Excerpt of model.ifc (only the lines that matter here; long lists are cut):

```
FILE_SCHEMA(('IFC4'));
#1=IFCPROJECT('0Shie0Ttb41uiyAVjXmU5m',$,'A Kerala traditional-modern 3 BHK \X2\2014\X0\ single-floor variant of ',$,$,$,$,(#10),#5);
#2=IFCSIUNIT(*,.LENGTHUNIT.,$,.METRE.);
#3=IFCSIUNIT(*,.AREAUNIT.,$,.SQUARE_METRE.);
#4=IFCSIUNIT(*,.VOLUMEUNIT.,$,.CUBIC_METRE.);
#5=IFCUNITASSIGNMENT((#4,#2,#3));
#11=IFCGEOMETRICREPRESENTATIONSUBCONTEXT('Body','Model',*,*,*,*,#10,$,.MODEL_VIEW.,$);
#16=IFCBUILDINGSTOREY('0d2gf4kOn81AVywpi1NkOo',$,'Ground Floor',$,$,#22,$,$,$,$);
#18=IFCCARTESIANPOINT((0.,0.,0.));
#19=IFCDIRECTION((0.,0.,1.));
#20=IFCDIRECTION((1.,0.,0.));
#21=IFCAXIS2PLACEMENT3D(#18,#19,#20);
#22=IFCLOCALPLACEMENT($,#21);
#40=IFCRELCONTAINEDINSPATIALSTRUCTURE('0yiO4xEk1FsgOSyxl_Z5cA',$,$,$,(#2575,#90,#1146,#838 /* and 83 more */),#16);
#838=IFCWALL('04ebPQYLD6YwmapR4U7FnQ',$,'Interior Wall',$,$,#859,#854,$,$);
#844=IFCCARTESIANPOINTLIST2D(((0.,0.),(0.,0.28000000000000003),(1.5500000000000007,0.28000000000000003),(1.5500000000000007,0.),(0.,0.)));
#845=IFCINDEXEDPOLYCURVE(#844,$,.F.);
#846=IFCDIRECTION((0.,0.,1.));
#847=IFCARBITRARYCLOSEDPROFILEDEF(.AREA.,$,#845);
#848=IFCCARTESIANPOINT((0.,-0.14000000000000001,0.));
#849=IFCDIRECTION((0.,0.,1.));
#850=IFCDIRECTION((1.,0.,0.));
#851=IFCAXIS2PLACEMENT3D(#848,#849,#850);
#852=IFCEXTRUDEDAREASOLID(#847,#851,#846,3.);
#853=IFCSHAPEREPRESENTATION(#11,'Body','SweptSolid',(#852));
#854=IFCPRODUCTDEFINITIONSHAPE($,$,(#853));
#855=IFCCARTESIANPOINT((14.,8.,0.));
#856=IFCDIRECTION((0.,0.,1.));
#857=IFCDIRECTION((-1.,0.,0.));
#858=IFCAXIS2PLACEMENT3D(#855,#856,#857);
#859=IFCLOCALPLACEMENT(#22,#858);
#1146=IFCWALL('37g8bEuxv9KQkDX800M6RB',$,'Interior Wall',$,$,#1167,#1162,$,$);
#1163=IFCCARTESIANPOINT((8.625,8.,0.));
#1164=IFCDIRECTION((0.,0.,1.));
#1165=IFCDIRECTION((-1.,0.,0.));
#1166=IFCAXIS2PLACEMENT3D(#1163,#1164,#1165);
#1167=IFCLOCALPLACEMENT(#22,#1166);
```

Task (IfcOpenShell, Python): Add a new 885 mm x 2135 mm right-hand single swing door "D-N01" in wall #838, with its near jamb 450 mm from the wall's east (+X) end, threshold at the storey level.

```python
import numpy as np
import ifcopenshell
import ifcopenshell.api.feature
import ifcopenshell.api.geometry
import ifcopenshell.api.root
import ifcopenshell.api.spatial
import ifcopenshell.geom
import ifcopenshell.util.element
import ifcopenshell.util.placement
import ifcopenshell.util.representation
import ifcopenshell.util.shape
import ifcopenshell.util.unit

model = ifcopenshell.open("model.ifc")
unit_scale = ifcopenshell.util.unit.calculate_unit_scale(model)
settings = ifcopenshell.geom.settings()


def volume(element):
    """Net volume in cubic metres, openings subtracted."""
    shape = ifcopenshell.geom.create_shape(settings, element)
    return ifcopenshell.util.shape.get_volume(shape.geometry)


wall = model.by_guid("04ebPQYLD6YwmapR4U7FnQ")
storey = ifcopenshell.util.element.get_container(wall, ifc_class="IfcBuildingStorey")
context = ifcopenshell.util.representation.get_context(model, "Model", "Body", "MODEL_VIEW")
before = volume(wall)

width, height, from_end, sill = 0.885, 2.135, 0.45, 0.0  # metres

# The wall runs along its own X axis, and the end named is its -X end.
wall_shape = ifcopenshell.geom.create_shape(settings, wall)
x, y, z = ifcopenshell.util.shape.get_vertices(wall_shape.geometry).T
start = x.min() + from_end
face, thickness = float(y.min()), float(y.max() - y.min())
wall_matrix = ifcopenshell.util.placement.get_local_placement(wall.ObjectPlacement)
level = ifcopenshell.util.placement.get_local_placement(storey.ObjectPlacement)[2, 3]


def in_wall(x, y):
    """Placement at x, y metres in the wall's axes, at sill height."""
    matrix = wall_matrix.copy()
    matrix[:, 3] = wall_matrix @ np.array([x / unit_scale, y / unit_scale, 0.0, 1.0])
    matrix[2, 3] = level + sill / unit_scale
    return matrix


# Opening: a box that overshoots both wall faces by 50 mm.
opening = ifcopenshell.api.root.create_entity(model, ifc_class="IfcOpeningElement", predefined_type="OPENING")
box = ifcopenshell.api.geometry.add_wall_representation(
    model, context=context, length=width, height=height, thickness=thickness + 0.1
)
ifcopenshell.api.geometry.assign_representation(model, product=opening, representation=box)
ifcopenshell.api.geometry.edit_object_placement(model, product=opening, matrix=in_wall(start, face - 0.05), is_si=False)
ifcopenshell.api.feature.add_feature(model, feature=opening, element=wall)

door = ifcopenshell.api.root.create_entity(model, ifc_class="IfcDoor", name="D-N01", predefined_type="DOOR")
door.OverallWidth, door.OverallHeight = width / unit_scale, height / unit_scale
door.OperationType = "SINGLE_SWING_RIGHT"
body = ifcopenshell.api.geometry.add_door_representation(
    model,
    context=context,
    overall_width=door.OverallWidth,
    overall_height=door.OverallHeight,
    operation_type="SINGLE_SWING_RIGHT",
    lining_properties={"LiningDepth": thickness / unit_scale, "ThresholdDepth": thickness / unit_scale},
)
ifcopenshell.api.geometry.assign_representation(model, product=door, representation=body)
ifcopenshell.api.spatial.assign_container(model, products=[door], relating_structure=storey)
ifcopenshell.api.feature.add_filling(model, opening=opening, element=door)

# The lining spans the wall, so the door starts at the wall face.
ifcopenshell.api.geometry.edit_object_placement(model, product=door, matrix=in_wall(start, face), is_si=False)

after = volume(wall)

print(f"wall volume {before:.3f} -> {after:.3f} m3")

model.write("model-out.ifc")
```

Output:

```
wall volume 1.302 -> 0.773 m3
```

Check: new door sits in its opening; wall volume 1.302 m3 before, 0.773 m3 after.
